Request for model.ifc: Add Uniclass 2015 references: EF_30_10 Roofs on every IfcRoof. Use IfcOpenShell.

First a look at what the model holds.

```python
import ifcopenshell

model = ifcopenshell.open("model.ifc")
print(model.schema)
print("classifications:", [c.Name for c in model.by_type("IfcClassification")])
for ifc_class in ("IfcDoor", "IfcRoof", "IfcStair", "IfcWall", "IfcWindow"):
    print(ifc_class, len(model.by_type(ifc_class)))
```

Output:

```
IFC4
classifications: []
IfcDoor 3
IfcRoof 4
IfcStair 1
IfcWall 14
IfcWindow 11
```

```python
import ifcopenshell
import ifcopenshell.api.classification

model = ifcopenshell.open("model.ifc")

system = ifcopenshell.api.classification.add_classification(model, classification="Uniclass 2015")

codes = {
    "IfcRoof": ("EF_30_10", "Roofs"),
}
for ifc_class, (code, name) in codes.items():
    products = model.by_type(ifc_class)
    ifcopenshell.api.classification.add_reference(
        model, products=products, classification=system, identification=code, name=name
    )
    print(code, len(products))

model.write("model_v2.ifc")
```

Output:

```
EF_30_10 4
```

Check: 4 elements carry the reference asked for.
